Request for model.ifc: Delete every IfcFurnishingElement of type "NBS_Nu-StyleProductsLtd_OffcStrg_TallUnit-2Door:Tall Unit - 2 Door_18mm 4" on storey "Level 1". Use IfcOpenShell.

First a look at what the model holds.

```python
import ifcopenshell
import ifcopenshell.util.element

model = ifcopenshell.open("model.ifc")
print(model.schema)
storey = next(s for s in model.by_type("IfcBuildingStorey") if s.Name == "Level 1")
furniture = [e for e in ifcopenshell.util.element.get_decomposition(storey) if e.is_a("IfcFurnishingElement")]
seen = {}
for e in furniture:
    element_type = ifcopenshell.util.element.get_type(e)
    name = element_type.Name if element_type not in (None, e) else None
    seen[name] = seen.get(name, 0) + 1
for name, count in sorted(seen.items(), key=str):
    print(count, "x", name)
```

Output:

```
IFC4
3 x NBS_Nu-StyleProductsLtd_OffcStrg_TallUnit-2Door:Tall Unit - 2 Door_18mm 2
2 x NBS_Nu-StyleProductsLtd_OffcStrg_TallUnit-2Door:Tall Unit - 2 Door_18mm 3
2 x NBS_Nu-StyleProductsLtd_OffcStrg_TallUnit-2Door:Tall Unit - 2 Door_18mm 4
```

```python
import ifcopenshell
import ifcopenshell.api.root
import ifcopenshell.util.element

model = ifcopenshell.open("model.ifc")

storey = next(s for s in model.by_type("IfcBuildingStorey") if s.Name == "Level 1")
furniture = [e for e in ifcopenshell.util.element.get_decomposition(storey) if e.is_a("IfcFurnishingElement")]
targets = [e for e in furniture if (t := ifcopenshell.util.element.get_type(e)) not in (None, e) and t.Name == "NBS_Nu-StyleProductsLtd_OffcStrg_TallUnit-2Door:Tall Unit - 2 Door_18mm 4"]

for e in targets:
    ifcopenshell.api.root.remove_product(model, product=e)
print(len(targets), "removed")

model.write("model_updated.ifc")
```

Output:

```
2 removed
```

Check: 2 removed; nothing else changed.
